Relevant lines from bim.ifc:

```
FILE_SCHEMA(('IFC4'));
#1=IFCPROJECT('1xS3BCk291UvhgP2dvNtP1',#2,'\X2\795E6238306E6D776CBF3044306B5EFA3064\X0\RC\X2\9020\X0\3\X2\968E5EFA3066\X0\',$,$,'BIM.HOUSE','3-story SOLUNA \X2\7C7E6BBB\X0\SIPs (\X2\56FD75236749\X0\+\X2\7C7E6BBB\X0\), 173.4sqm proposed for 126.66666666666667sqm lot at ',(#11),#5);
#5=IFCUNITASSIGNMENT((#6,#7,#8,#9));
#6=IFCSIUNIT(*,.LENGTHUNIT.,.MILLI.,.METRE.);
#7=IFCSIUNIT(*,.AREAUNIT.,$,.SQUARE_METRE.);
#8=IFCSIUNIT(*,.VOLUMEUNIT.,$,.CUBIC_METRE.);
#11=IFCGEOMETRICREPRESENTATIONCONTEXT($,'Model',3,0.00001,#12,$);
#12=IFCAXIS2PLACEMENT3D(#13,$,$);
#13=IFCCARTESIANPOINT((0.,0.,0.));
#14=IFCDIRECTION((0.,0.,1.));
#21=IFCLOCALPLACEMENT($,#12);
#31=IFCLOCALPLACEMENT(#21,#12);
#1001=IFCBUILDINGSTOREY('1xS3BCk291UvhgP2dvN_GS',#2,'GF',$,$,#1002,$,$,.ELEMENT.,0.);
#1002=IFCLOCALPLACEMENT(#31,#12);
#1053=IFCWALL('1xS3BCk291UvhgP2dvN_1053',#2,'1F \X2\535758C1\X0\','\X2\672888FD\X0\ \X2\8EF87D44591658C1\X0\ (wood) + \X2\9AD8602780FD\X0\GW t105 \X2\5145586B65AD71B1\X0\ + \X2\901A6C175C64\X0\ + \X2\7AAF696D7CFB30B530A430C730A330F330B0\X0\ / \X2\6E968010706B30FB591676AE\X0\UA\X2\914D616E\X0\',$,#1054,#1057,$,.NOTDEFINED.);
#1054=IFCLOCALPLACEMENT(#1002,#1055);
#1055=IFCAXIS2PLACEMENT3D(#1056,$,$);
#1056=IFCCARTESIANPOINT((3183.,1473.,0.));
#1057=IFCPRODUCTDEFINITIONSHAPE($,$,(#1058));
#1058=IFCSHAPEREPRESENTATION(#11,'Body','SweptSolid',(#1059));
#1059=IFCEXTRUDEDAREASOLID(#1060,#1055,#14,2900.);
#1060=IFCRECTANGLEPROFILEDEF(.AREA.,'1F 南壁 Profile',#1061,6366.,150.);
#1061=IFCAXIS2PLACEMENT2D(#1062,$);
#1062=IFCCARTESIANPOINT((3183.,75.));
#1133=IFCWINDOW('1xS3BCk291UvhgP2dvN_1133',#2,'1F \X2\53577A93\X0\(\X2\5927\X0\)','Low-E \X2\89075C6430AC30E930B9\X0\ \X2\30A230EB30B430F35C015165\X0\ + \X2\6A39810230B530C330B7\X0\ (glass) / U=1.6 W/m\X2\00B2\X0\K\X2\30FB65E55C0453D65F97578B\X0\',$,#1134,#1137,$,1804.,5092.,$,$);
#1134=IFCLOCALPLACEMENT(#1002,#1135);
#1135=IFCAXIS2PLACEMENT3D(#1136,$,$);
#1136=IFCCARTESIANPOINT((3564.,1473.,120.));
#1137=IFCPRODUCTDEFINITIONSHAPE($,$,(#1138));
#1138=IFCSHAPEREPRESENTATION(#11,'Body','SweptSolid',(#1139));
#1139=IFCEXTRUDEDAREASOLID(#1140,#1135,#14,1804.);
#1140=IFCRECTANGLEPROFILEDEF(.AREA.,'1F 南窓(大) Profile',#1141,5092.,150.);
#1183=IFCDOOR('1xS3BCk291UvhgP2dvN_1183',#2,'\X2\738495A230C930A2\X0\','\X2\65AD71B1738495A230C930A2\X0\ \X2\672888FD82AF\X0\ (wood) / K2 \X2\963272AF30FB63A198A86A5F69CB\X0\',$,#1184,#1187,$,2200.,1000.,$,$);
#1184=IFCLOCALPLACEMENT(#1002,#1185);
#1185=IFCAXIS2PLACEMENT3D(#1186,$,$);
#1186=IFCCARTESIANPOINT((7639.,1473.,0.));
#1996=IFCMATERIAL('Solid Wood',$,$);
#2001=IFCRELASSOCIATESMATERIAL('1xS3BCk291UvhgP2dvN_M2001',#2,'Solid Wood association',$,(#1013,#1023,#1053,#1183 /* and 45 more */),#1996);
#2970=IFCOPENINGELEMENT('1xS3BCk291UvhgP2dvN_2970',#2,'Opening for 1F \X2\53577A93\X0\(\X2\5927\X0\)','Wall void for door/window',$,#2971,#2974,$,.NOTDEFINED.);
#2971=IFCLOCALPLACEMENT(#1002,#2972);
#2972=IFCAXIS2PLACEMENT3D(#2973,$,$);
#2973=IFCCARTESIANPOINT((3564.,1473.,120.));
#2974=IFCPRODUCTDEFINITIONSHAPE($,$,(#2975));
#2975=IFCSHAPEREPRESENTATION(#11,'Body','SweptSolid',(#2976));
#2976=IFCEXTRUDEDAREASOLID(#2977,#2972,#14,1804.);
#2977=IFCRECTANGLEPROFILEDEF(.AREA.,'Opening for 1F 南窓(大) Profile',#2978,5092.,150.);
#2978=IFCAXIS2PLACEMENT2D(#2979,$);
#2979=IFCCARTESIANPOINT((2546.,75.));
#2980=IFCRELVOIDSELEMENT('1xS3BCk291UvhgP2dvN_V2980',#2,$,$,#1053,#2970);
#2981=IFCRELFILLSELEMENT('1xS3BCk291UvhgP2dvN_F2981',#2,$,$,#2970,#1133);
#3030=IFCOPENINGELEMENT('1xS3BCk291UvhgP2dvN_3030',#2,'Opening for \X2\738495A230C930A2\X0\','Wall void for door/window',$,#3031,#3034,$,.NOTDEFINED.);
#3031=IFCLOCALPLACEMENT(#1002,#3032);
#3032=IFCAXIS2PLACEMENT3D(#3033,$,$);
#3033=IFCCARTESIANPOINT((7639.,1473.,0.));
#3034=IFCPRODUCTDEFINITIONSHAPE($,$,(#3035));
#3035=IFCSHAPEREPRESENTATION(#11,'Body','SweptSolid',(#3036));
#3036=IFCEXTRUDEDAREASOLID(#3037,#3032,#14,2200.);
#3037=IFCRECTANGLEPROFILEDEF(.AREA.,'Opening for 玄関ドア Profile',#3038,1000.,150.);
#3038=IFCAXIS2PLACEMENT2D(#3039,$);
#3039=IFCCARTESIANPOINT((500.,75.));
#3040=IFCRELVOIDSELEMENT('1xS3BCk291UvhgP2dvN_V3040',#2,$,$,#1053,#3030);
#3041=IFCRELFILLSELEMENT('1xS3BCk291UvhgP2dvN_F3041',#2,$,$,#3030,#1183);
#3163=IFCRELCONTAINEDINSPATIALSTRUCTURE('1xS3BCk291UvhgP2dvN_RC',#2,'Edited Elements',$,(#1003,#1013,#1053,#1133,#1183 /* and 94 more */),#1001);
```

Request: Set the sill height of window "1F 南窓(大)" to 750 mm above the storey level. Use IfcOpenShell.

```python
import numpy as np
import ifcopenshell
import ifcopenshell.api.geometry
import ifcopenshell.geom
import ifcopenshell.util.element
import ifcopenshell.util.placement
import ifcopenshell.util.shape
import ifcopenshell.util.unit

model = ifcopenshell.open("bim.ifc")
unit_scale = ifcopenshell.util.unit.calculate_unit_scale(model)

window = model.by_guid("1xS3BCk291UvhgP2dvN_1133")
opening = window.FillsVoids[0].RelatingOpeningElement
storey = ifcopenshell.util.element.get_container(window, ifc_class="IfcBuildingStorey")
level = ifcopenshell.util.placement.get_local_placement(storey.ObjectPlacement)[2, 3]

# The opening's origin need not be at the sill, so measure its lowest point.
shape = ifcopenshell.geom.create_shape(ifcopenshell.geom.settings(), opening)
bottom = ifcopenshell.util.shape.get_shape_bottom_elevation(shape, shape.geometry) / unit_scale
dz = level + 750.0 - bottom

shift = np.array([0.0, 0.0, dz])
# The window is not placed relative to its opening, so move both.
for product in (opening, window):
    matrix = ifcopenshell.util.placement.get_local_placement(product.ObjectPlacement)
    matrix[:3, 3] += shift
    ifcopenshell.api.geometry.edit_object_placement(model, product=product, matrix=matrix, is_si=False)

print(f"moved by {dz * unit_scale:+.3f} m")

model.write("bim_v2.ifc")
```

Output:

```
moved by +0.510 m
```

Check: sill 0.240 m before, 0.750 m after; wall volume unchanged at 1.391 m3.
